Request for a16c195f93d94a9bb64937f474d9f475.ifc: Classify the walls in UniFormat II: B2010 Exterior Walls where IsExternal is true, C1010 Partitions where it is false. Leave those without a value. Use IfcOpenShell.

First a look at what the model holds.

```python
import ifcopenshell
import ifcopenshell.util.element

model = ifcopenshell.open("a16c195f93d94a9bb64937f474d9f475.ifc")
print(model.schema)
print("classifications:", [c.Name for c in model.by_type("IfcClassification")])
values = [ifcopenshell.util.element.get_pset(e, "Pset_WallCommon", "IsExternal") for e in model.by_type("IfcWall")]
for value in (True, False, None):
    print("IsExternal", value, values.count(value))
```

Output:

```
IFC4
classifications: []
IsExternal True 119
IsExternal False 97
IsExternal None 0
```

```python
import ifcopenshell
import ifcopenshell.api.classification
import ifcopenshell.util.element

model = ifcopenshell.open("a16c195f93d94a9bb64937f474d9f475.ifc")

system = ifcopenshell.api.classification.add_classification(model, classification="UniFormat II")

walls = model.by_type("IfcWall")
external = {e: ifcopenshell.util.element.get_pset(e, "Pset_WallCommon", "IsExternal") for e in walls}
for flag, code, name in ((True, "B2010", "Exterior Walls"), (False, "C1010", "Partitions")):
    products = [e for e in walls if external[e] is flag]
    ifcopenshell.api.classification.add_reference(
        model, products=products, classification=system, identification=code, name=name
    )
    print(code, len(products))

model.write("a16c195f93d94a9bb64937f474d9f475_edited.ifc")
```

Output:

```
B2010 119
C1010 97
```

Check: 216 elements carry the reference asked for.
